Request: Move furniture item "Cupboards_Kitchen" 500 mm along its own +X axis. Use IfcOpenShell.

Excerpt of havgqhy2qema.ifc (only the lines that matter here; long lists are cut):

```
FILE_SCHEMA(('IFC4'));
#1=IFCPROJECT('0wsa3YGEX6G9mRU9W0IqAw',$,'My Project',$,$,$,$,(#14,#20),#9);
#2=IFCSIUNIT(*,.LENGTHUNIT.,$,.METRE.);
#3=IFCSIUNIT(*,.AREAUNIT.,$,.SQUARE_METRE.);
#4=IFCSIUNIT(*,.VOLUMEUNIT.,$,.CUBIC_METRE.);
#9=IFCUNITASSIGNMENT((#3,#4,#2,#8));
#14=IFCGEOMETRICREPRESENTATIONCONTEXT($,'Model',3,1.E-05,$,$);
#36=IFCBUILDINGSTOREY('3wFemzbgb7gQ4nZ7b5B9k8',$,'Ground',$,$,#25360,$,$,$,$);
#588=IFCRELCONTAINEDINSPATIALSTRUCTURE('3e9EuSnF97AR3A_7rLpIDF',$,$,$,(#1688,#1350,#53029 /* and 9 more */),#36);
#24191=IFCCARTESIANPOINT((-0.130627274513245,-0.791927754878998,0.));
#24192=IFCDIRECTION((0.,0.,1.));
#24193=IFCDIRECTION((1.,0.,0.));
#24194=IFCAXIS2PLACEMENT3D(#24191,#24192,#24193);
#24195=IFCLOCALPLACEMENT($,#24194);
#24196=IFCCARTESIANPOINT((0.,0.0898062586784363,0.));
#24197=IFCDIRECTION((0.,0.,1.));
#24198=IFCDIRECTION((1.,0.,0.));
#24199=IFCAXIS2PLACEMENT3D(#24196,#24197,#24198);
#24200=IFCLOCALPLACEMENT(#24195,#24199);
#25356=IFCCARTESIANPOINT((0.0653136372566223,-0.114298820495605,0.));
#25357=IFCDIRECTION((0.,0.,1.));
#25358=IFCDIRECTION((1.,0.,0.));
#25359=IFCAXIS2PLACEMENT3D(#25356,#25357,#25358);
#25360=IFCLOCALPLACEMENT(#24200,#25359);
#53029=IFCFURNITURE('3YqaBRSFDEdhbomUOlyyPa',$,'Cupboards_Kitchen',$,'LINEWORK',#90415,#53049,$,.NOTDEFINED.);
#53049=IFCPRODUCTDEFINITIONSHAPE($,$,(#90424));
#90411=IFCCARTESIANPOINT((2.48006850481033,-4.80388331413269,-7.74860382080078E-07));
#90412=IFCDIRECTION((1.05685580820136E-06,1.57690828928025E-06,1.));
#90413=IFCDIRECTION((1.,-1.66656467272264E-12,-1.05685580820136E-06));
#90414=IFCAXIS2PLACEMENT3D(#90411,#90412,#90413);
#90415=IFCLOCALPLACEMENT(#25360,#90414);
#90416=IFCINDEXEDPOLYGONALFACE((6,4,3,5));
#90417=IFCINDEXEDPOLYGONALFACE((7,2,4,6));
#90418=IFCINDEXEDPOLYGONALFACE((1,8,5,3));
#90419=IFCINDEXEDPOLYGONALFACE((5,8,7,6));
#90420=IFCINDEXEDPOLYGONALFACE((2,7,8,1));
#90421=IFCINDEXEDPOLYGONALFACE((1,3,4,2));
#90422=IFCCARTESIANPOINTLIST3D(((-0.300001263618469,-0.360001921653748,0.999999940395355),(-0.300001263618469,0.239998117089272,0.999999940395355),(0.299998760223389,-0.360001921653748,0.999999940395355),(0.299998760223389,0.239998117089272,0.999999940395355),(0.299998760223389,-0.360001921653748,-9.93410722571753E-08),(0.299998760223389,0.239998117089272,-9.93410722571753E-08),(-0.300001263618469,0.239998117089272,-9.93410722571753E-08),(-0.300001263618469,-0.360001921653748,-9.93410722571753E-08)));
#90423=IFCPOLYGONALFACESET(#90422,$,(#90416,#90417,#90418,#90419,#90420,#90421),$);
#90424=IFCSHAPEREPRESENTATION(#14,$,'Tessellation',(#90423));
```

```python
import ifcopenshell
import ifcopenshell.api.geometry
import ifcopenshell.util.placement
import ifcopenshell.util.unit

model = ifcopenshell.open("havgqhy2qema.ifc")
unit_scale = ifcopenshell.util.unit.calculate_unit_scale(model)

item = model.by_guid("3YqaBRSFDEdhbomUOlyyPa")
matrix = ifcopenshell.util.placement.get_local_placement(item.ObjectPlacement)
matrix[:3, 3] += matrix[:3, 0] * 0.5 / unit_scale
ifcopenshell.api.geometry.edit_object_placement(model, product=item, matrix=matrix, is_si=False)

print(ifcopenshell.util.placement.get_local_placement(item.ObjectPlacement).round(3) + 0.0)

model.write("havgqhy2qema_edited.ifc")
```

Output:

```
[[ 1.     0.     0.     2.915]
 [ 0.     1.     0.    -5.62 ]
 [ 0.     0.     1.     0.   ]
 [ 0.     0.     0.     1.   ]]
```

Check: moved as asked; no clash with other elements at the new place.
